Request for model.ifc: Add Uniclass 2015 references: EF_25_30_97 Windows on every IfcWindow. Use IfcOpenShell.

First a look at what the model holds.

```python
import ifcopenshell

model = ifcopenshell.open("model.ifc")
print(model.schema)
print("classifications:", [c.Name for c in model.by_type("IfcClassification")])
for ifc_class in ("IfcDoor", "IfcRoof", "IfcStair", "IfcWall", "IfcWindow"):
    print(ifc_class, len(model.by_type(ifc_class)))
```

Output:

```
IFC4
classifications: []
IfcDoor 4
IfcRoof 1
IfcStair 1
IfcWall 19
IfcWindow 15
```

```python
import ifcopenshell
import ifcopenshell.api.classification

model = ifcopenshell.open("model.ifc")

system = ifcopenshell.api.classification.add_classification(model, classification="Uniclass 2015")

codes = {
    "IfcWindow": ("EF_25_30_97", "Windows"),
}
for ifc_class, (code, name) in codes.items():
    products = model.by_type(ifc_class)
    ifcopenshell.api.classification.add_reference(
        model, products=products, classification=system, identification=code, name=name
    )
    print(code, len(products))

model.write("model_updated.ifc")
```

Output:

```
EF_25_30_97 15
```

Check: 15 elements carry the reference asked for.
